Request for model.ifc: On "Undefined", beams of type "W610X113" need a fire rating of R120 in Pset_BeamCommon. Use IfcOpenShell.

First a look at what the model holds.

```python
import ifcopenshell
import ifcopenshell.util.element

model = ifcopenshell.open("model.ifc")
print(model.schema)
storey = next(s for s in model.by_type("IfcBuildingStorey") if s.Name == "Undefined")
beams = [e for e in ifcopenshell.util.element.get_decomposition(storey) if e.is_a("IfcBeam")]
seen = {}
for e in beams:
    element_type = ifcopenshell.util.element.get_type(e)
    key = (element_type.Name if element_type != e and element_type else None, ifcopenshell.util.element.get_pset(e, "Pset_BeamCommon", "FireRating"))
    seen[key] = seen.get(key, 0) + 1
for (name, value), count in sorted(seen.items(), key=str):
    print(count, "x", name, "|", value)
```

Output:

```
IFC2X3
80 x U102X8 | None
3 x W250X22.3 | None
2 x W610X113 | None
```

```python
import ifcopenshell
import ifcopenshell.api.pset
import ifcopenshell.util.element

model = ifcopenshell.open("model.ifc")

storey = next(s for s in model.by_type("IfcBuildingStorey") if s.Name == "Undefined")
beams = [e for e in ifcopenshell.util.element.get_decomposition(storey) if e.is_a("IfcBeam")]

count = 0
for e in beams:
    element_type = ifcopenshell.util.element.get_type(e)
    if element_type in (None, e) or element_type.Name != "W610X113":
        continue
    found = ifcopenshell.util.element.get_pset(e, "Pset_BeamCommon", should_inherit=False)
    if found:
        pset = model.by_id(found["id"])
        if len(ifcopenshell.util.element.get_elements_by_pset(pset)) > 1:
            pset = ifcopenshell.api.pset.unshare_pset(model, products=[e], pset=pset)[0]
    else:
        pset = ifcopenshell.api.pset.add_pset(model, product=e, name="Pset_BeamCommon")
    ifcopenshell.api.pset.edit_pset(model, pset=pset, properties={"FireRating": "R120"})
    count += 1

print(count, "beams updated")

model.write("model_v2.ifc")
```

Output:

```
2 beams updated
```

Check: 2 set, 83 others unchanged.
